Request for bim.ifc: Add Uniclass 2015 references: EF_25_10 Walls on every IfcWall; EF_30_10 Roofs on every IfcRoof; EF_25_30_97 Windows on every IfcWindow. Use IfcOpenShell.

First a look at what the model holds.

```python
import ifcopenshell

model = ifcopenshell.open("bim.ifc")
print(model.schema)
print("classifications:", [c.Name for c in model.by_type("IfcClassification")])
for ifc_class in ("IfcDoor", "IfcRoof", "IfcStair", "IfcWall", "IfcWindow"):
    print(ifc_class, len(model.by_type(ifc_class)))
```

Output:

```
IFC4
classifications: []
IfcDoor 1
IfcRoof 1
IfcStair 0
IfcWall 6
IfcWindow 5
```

```python
import ifcopenshell
import ifcopenshell.api.classification

model = ifcopenshell.open("bim.ifc")

system = ifcopenshell.api.classification.add_classification(model, classification="Uniclass 2015")

codes = {
    "IfcWall": ("EF_25_10", "Walls"),
    "IfcRoof": ("EF_30_10", "Roofs"),
    "IfcWindow": ("EF_25_30_97", "Windows"),
}
for ifc_class, (code, name) in codes.items():
    products = model.by_type(ifc_class)
    ifcopenshell.api.classification.add_reference(
        model, products=products, classification=system, identification=code, name=name
    )
    print(code, len(products))

model.write("bim-out.ifc")
```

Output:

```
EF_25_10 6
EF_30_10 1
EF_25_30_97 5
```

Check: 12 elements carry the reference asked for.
